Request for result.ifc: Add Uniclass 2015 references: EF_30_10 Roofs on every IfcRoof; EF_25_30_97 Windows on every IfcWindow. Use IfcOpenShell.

First a look at what the model holds.

```python
import ifcopenshell

model = ifcopenshell.open("result.ifc")
print(model.schema)
print("classifications:", [c.Name for c in model.by_type("IfcClassification")])
for ifc_class in ("IfcDoor", "IfcRoof", "IfcStair", "IfcWall", "IfcWindow"):
    print(ifc_class, len(model.by_type(ifc_class)))
```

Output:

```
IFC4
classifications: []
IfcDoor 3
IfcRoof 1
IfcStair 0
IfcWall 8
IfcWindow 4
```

```python
import ifcopenshell
import ifcopenshell.api.classification

model = ifcopenshell.open("result.ifc")

system = ifcopenshell.api.classification.add_classification(model, classification="Uniclass 2015")

codes = {
    "IfcRoof": ("EF_30_10", "Roofs"),
    "IfcWindow": ("EF_25_30_97", "Windows"),
}
for ifc_class, (code, name) in codes.items():
    products = model.by_type(ifc_class)
    ifcopenshell.api.classification.add_reference(
        model, products=products, classification=system, identification=code, name=name
    )
    print(code, len(products))

model.write("result_updated.ifc")
```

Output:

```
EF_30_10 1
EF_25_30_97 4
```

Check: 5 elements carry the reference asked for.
